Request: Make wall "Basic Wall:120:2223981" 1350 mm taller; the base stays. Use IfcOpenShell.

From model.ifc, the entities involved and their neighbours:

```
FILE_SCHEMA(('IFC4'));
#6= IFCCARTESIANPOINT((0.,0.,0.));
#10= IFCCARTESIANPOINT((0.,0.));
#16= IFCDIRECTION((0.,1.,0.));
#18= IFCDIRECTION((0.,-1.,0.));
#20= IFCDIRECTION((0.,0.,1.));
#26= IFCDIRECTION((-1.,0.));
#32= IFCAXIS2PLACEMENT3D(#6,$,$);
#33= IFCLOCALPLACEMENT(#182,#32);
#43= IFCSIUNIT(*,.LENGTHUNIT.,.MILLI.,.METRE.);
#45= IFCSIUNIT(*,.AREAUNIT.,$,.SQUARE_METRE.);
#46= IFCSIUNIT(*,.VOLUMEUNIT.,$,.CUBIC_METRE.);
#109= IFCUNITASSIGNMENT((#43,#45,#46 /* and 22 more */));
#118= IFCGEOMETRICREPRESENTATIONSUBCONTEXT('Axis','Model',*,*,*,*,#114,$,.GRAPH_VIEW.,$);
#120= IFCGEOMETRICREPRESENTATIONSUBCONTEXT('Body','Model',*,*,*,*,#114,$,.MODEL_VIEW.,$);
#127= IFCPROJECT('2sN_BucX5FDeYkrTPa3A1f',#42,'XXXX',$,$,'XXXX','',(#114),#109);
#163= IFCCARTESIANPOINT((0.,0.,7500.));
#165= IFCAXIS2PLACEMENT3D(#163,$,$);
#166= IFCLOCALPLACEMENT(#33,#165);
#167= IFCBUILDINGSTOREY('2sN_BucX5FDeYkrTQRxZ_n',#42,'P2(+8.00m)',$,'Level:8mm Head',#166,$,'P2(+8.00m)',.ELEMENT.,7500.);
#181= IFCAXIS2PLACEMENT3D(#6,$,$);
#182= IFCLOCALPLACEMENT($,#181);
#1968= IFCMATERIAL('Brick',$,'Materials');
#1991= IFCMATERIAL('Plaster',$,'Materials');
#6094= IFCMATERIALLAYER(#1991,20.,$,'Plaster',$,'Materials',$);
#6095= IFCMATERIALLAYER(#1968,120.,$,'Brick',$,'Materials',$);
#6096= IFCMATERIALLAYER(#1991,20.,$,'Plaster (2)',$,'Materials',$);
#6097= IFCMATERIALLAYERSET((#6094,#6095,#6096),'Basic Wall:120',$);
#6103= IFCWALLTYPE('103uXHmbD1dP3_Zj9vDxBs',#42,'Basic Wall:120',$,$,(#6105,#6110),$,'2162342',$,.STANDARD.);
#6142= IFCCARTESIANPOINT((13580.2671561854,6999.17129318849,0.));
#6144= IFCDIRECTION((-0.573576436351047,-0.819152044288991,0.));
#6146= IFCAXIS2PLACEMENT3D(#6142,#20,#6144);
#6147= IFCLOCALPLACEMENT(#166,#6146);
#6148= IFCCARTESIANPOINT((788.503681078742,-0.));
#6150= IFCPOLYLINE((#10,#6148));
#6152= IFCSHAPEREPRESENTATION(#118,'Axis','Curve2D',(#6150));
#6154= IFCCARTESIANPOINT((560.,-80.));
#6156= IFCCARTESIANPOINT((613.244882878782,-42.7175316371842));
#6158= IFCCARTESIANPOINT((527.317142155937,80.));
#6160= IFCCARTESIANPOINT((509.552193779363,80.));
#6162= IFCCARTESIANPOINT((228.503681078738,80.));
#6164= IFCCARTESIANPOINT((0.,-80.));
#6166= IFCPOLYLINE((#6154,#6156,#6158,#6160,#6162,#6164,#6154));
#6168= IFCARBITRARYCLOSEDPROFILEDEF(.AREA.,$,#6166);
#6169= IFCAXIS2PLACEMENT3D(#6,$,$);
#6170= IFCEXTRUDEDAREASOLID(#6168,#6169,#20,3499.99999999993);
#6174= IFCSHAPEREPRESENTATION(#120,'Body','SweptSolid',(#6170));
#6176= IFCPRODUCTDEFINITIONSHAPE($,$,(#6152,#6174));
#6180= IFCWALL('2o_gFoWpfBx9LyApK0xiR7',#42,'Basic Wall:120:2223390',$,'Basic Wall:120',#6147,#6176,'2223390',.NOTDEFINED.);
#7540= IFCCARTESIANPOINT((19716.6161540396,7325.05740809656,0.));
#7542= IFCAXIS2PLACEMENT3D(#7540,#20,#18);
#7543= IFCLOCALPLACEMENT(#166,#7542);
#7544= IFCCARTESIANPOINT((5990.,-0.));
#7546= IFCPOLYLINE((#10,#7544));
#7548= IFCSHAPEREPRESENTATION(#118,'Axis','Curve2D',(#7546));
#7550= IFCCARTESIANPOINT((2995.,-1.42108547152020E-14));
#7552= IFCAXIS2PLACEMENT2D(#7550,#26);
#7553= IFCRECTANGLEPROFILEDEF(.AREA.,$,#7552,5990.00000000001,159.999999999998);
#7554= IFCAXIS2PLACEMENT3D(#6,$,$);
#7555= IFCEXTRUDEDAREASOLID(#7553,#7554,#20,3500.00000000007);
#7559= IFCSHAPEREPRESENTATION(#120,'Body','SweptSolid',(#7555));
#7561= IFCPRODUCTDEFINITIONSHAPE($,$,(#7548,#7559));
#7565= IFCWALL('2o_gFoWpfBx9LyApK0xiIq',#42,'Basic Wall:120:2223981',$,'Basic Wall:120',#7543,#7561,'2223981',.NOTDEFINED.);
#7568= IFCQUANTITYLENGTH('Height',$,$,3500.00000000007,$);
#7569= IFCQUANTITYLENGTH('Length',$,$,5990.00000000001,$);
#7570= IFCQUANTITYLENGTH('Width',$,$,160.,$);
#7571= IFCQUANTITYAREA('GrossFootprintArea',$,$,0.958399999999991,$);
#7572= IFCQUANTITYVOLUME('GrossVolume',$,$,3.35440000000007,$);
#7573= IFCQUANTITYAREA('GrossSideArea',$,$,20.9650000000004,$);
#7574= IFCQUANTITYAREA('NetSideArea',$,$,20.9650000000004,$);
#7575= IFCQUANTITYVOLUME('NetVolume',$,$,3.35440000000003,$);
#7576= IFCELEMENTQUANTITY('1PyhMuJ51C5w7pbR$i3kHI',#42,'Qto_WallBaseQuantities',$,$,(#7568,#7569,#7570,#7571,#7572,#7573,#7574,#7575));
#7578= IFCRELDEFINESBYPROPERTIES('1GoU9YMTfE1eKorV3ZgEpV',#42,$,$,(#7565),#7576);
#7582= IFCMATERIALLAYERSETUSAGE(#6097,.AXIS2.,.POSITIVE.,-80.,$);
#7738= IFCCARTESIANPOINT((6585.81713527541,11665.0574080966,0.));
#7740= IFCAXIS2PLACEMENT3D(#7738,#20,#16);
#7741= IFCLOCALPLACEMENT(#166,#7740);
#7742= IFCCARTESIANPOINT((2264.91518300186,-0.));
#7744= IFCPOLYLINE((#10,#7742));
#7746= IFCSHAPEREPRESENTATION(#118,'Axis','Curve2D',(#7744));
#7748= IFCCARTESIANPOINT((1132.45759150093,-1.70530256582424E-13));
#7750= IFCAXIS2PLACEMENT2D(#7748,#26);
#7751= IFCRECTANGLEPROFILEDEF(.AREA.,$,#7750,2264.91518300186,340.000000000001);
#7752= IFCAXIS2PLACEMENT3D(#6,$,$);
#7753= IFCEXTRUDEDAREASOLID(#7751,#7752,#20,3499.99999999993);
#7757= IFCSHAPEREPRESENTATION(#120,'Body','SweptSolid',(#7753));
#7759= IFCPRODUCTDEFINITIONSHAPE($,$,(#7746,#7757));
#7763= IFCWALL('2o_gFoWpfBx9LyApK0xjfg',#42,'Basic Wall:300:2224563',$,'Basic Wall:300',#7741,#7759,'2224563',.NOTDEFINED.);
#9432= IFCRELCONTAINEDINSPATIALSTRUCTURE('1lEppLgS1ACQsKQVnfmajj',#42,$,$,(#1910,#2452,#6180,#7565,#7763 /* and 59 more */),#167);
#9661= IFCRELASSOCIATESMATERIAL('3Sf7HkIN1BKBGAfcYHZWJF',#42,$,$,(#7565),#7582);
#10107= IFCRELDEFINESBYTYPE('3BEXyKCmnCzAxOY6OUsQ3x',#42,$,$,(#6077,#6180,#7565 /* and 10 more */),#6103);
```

```python
import ifcopenshell
import ifcopenshell.api.pset
import ifcopenshell.geom
import ifcopenshell.util.element
import ifcopenshell.util.representation
import ifcopenshell.util.shape
import ifcopenshell.util.unit

model = ifcopenshell.open("model.ifc")
unit_scale = ifcopenshell.util.unit.calculate_unit_scale(model)
area_scale = ifcopenshell.util.unit.calculate_unit_scale(model, "AREAUNIT")
volume_scale = ifcopenshell.util.unit.calculate_unit_scale(model, "VOLUMEUNIT")
settings = ifcopenshell.geom.settings()


def volume(element):
    """Net volume in cubic metres, openings subtracted."""
    shape = ifcopenshell.geom.create_shape(settings, element)
    return ifcopenshell.util.shape.get_volume(shape.geometry)


wall = model.by_id(7565)
before = volume(wall)

body = ifcopenshell.util.representation.get_representation(wall, "Model", "Body")
solid = body.Items[0]
old_height = solid.Depth
solid.Depth += 1.35 / unit_scale
after = volume(wall)
thickness = 0.16  # wall thickness in metres

# Update the stored height, areas and volumes.
qto = model.by_id(ifcopenshell.util.element.get_pset(wall, "Qto_WallBaseQuantities", should_inherit=False)["id"])
ifcopenshell.api.pset.edit_qto(model, qto=qto, properties={
    "Height": solid.Depth,
    "GrossVolume": ifcopenshell.util.element.get_pset(wall, "Qto_WallBaseQuantities", "GrossVolume") * solid.Depth / old_height,
    "GrossSideArea": ifcopenshell.util.element.get_pset(wall, "Qto_WallBaseQuantities", "GrossSideArea") * solid.Depth / old_height,
    "NetSideArea": after / thickness / area_scale,
    "NetVolume": after / volume_scale,
})

print(f"height {old_height:g} -> {solid.Depth:g}, volume {before:.3f} -> {after:.3f} m3")

model.write("model-out.ifc")
```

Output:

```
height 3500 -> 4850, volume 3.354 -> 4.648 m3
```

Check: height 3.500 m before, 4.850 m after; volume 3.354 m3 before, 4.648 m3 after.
